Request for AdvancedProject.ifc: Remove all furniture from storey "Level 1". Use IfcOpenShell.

First a look at what the model holds.

```python
import ifcopenshell
import ifcopenshell.util.element

model = ifcopenshell.open("AdvancedProject.ifc")
print(model.schema)
storey = next(s for s in model.by_type("IfcBuildingStorey") if s.Name == "Level 1")
furniture = [e for e in ifcopenshell.util.element.get_decomposition(storey) if e.is_a("IfcFurnishingElement")]
seen = {}
for e in furniture:
    element_type = ifcopenshell.util.element.get_type(e)
    name = element_type.Name if element_type not in (None, e) else None
    seen[name] = seen.get(name, 0) + 1
for name, count in sorted(seen.items(), key=str):
    print(count, "x", name)
```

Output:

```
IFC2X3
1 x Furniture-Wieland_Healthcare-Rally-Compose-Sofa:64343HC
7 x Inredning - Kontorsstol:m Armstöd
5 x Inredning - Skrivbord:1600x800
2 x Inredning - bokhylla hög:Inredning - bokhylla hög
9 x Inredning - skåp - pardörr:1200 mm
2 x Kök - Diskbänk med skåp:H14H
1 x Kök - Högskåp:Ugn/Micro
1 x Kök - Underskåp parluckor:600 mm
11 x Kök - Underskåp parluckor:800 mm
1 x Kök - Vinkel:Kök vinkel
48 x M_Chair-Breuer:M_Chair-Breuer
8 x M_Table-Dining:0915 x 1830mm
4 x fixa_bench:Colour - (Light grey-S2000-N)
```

```python
import ifcopenshell
import ifcopenshell.api.root
import ifcopenshell.util.element

model = ifcopenshell.open("AdvancedProject.ifc")

storey = next(s for s in model.by_type("IfcBuildingStorey") if s.Name == "Level 1")
furniture = [e for e in ifcopenshell.util.element.get_decomposition(storey) if e.is_a("IfcFurnishingElement")]

for e in furniture:
    ifcopenshell.api.root.remove_product(model, product=e)
print(len(furniture), "removed")

model.write("AdvancedProject_updated.ifc")
```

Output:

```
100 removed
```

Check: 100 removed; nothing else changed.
